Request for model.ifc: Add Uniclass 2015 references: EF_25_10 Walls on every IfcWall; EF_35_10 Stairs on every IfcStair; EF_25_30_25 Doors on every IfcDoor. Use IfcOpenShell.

First a look at what the model holds.

```python
import ifcopenshell

model = ifcopenshell.open("model.ifc")
print(model.schema)
print("classifications:", [c.Name for c in model.by_type("IfcClassification")])
for ifc_class in ("IfcDoor", "IfcRoof", "IfcStair", "IfcWall", "IfcWindow"):
    print(ifc_class, len(model.by_type(ifc_class)))
```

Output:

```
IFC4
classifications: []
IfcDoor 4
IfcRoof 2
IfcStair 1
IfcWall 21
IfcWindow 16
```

```python
import ifcopenshell
import ifcopenshell.api.classification

model = ifcopenshell.open("model.ifc")

system = ifcopenshell.api.classification.add_classification(model, classification="Uniclass 2015")

codes = {
    "IfcWall": ("EF_25_10", "Walls"),
    "IfcStair": ("EF_35_10", "Stairs"),
    "IfcDoor": ("EF_25_30_25", "Doors"),
}
for ifc_class, (code, name) in codes.items():
    products = model.by_type(ifc_class)
    ifcopenshell.api.classification.add_reference(
        model, products=products, classification=system, identification=code, name=name
    )
    print(code, len(products))

model.write("model_rev.ifc")
```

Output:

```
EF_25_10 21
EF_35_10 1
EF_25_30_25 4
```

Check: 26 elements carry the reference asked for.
